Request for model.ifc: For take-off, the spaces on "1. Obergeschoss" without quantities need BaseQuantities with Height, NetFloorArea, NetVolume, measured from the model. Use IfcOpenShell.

First a look at what the model holds.

```python
import ifcopenshell
import ifcopenshell.util.element
import ifcopenshell.util.unit

model = ifcopenshell.open("model.ifc")
print(model.schema)
for unit_type in ("LENGTHUNIT", "AREAUNIT", "VOLUMEUNIT"):
    print(unit_type, ifcopenshell.util.unit.calculate_unit_scale(model, unit_type))
storey = next(s for s in model.by_type("IfcBuildingStorey") if s.Name == "1. Obergeschoss")
spaces = [e for e in ifcopenshell.util.element.get_decomposition(storey) if e.is_a("IfcSpace")]
for e in sorted(spaces, key=lambda e: e.id()):
    print(e.id(), e.is_a(), e.Name, list(ifcopenshell.util.element.get_psets(e, qtos_only=True)), sep=" | ")
```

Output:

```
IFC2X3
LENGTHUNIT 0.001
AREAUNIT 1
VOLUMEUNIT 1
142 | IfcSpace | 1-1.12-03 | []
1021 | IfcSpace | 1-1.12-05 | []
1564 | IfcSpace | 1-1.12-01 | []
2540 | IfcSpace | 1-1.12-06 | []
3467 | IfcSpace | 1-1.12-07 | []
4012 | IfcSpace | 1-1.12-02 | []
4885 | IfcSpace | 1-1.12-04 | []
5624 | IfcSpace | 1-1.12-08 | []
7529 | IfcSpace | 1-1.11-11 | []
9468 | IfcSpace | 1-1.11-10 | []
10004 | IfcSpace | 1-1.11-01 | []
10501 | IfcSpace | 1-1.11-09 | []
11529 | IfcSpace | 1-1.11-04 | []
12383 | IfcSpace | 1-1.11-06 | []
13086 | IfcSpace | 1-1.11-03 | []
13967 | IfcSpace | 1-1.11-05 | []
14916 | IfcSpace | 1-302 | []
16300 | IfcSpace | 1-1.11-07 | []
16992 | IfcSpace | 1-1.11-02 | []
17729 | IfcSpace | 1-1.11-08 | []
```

```python
import ifcopenshell
import ifcopenshell.api.pset
import ifcopenshell.geom
import ifcopenshell.util.element
import ifcopenshell.util.shape
import ifcopenshell.util.unit

model = ifcopenshell.open("model.ifc")
unit_scale = ifcopenshell.util.unit.calculate_unit_scale(model)
area_scale = ifcopenshell.util.unit.calculate_unit_scale(model, "AREAUNIT")
volume_scale = ifcopenshell.util.unit.calculate_unit_scale(model, "VOLUMEUNIT")
settings = ifcopenshell.geom.settings()

storey = next(s for s in model.by_type("IfcBuildingStorey") if s.Name == "1. Obergeschoss")
spaces = [e for e in ifcopenshell.util.element.get_decomposition(storey) if e.is_a("IfcSpace")]

for e in sorted(spaces, key=lambda e: e.id()):
    if ifcopenshell.util.element.get_psets(e, qtos_only=True, should_inherit=False):
        continue
    # Geometry comes back in metres, in the element's own axes.
    shape = ifcopenshell.geom.create_shape(settings, e)
    values = {
        "Height": ifcopenshell.util.shape.get_z(shape.geometry) / unit_scale,
        "NetFloorArea": ifcopenshell.util.shape.get_footprint_area(shape.geometry) / area_scale,
        "NetVolume": ifcopenshell.util.shape.get_volume(shape.geometry) / volume_scale,
    }
    qto = ifcopenshell.api.pset.add_qto(model, product=e, name="BaseQuantities")
    ifcopenshell.api.pset.edit_qto(model, qto=qto, properties=values)
    print(e.id(), {k: round(v, 3) for k, v in values.items()})

model.write("model-out.ifc")
```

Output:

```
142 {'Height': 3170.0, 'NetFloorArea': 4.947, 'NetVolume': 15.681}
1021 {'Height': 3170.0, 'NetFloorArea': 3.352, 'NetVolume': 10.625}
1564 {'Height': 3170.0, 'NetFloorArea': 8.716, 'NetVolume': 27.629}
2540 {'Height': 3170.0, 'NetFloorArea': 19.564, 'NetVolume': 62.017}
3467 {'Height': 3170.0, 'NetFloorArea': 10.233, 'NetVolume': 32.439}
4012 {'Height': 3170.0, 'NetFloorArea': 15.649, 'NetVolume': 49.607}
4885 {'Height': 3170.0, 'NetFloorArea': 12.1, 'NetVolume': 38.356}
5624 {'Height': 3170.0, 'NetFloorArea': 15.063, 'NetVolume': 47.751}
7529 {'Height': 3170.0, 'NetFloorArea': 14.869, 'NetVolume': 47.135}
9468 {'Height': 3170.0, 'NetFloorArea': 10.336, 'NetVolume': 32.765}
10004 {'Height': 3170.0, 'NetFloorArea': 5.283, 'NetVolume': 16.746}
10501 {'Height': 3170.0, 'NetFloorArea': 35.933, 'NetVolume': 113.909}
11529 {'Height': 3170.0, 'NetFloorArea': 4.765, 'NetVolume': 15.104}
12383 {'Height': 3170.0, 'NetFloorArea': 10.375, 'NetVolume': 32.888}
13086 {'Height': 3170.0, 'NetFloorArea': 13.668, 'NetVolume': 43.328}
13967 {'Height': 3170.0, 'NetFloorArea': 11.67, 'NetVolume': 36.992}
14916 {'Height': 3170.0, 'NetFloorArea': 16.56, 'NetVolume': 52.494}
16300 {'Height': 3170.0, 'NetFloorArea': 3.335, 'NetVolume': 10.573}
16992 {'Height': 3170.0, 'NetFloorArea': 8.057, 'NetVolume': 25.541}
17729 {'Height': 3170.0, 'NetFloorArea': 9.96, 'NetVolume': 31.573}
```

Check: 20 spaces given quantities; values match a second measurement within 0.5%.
